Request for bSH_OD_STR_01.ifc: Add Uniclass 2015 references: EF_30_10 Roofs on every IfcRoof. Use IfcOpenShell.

First a look at what the model holds.

```python
import ifcopenshell

model = ifcopenshell.open("bSH_OD_STR_01.ifc")
print(model.schema)
print("classifications:", [c.Name for c in model.by_type("IfcClassification")])
for ifc_class in ("IfcDoor", "IfcRoof", "IfcStair", "IfcWall", "IfcWindow"):
    print(ifc_class, len(model.by_type(ifc_class)))
```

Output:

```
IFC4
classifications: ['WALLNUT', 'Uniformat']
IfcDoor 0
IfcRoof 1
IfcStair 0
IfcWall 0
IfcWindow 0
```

```python
import ifcopenshell
import ifcopenshell.api.classification

model = ifcopenshell.open("bSH_OD_STR_01.ifc")

system = ifcopenshell.api.classification.add_classification(model, classification="Uniclass 2015")

codes = {
    "IfcRoof": ("EF_30_10", "Roofs"),
}
for ifc_class, (code, name) in codes.items():
    products = model.by_type(ifc_class)
    ifcopenshell.api.classification.add_reference(
        model, products=products, classification=system, identification=code, name=name
    )
    print(code, len(products))

model.write("bSH_OD_STR_01-out.ifc")
```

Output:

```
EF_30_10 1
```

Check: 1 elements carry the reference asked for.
